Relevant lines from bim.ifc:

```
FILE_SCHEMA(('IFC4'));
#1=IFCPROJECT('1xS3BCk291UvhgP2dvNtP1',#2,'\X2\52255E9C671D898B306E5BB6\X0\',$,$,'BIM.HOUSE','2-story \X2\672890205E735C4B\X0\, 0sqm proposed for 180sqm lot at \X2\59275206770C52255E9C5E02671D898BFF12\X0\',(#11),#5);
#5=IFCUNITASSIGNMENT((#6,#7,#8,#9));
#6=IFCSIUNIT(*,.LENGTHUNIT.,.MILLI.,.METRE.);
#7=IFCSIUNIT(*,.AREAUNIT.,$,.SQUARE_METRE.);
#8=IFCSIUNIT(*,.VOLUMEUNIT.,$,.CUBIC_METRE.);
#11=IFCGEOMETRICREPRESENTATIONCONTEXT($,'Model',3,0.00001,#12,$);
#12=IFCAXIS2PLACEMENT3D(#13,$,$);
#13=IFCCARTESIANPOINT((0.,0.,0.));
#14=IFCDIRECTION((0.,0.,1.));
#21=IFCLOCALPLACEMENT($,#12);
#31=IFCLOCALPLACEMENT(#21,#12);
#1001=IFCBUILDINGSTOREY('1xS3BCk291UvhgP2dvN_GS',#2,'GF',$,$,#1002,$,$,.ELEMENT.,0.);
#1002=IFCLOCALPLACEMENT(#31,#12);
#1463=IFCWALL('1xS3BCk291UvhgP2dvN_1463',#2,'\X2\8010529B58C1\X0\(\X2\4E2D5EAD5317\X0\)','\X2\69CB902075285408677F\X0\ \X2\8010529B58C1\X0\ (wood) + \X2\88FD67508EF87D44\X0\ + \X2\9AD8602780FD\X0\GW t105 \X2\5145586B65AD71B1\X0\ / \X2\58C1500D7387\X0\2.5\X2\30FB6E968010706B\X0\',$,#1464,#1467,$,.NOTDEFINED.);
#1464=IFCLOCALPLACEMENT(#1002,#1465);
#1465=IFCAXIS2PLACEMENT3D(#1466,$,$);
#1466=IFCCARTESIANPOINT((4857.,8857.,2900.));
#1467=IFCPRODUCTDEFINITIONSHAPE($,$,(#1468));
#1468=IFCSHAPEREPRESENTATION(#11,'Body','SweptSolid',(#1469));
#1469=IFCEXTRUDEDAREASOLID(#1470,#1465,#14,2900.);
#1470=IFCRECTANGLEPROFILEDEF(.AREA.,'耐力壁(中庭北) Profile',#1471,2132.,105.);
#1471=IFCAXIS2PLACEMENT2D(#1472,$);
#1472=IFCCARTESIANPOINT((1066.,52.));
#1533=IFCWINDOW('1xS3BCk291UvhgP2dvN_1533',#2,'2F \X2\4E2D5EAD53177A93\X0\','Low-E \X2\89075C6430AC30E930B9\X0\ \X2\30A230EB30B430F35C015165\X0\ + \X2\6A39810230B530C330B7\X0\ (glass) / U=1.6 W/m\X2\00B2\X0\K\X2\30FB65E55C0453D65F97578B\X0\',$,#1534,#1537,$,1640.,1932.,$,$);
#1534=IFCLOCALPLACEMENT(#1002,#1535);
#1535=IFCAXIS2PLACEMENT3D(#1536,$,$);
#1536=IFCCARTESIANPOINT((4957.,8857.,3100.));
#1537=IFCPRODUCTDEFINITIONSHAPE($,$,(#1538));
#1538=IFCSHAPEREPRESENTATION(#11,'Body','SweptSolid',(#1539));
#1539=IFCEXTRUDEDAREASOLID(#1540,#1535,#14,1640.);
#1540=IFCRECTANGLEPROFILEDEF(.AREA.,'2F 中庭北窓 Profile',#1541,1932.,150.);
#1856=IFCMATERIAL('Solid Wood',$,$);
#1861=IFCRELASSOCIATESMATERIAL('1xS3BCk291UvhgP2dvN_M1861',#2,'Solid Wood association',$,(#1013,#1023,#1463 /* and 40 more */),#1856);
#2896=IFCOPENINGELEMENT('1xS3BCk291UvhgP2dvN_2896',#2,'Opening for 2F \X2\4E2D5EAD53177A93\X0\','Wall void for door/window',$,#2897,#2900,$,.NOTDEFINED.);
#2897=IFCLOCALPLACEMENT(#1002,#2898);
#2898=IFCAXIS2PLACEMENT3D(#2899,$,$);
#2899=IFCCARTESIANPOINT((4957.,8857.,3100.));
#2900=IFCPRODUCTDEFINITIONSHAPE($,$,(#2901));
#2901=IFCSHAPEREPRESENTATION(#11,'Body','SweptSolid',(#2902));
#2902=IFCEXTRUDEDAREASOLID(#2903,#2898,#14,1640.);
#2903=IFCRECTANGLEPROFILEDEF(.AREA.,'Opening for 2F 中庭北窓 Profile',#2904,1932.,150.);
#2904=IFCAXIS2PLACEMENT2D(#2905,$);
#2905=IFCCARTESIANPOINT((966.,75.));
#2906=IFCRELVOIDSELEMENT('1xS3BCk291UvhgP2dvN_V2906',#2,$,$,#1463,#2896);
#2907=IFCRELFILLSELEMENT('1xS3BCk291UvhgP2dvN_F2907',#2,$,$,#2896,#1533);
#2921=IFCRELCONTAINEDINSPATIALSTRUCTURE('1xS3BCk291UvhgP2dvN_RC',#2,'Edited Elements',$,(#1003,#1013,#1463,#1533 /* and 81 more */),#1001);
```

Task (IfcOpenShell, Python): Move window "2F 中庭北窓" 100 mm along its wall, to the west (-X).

```python
import ifcopenshell
import ifcopenshell.api.geometry
import ifcopenshell.util.placement
import ifcopenshell.util.unit

model = ifcopenshell.open("bim.ifc")
unit_scale = ifcopenshell.util.unit.calculate_unit_scale(model)

window = model.by_guid("1xS3BCk291UvhgP2dvN_1533")
opening = window.FillsVoids[0].RelatingOpeningElement
wall = opening.VoidsElements[0].RelatingBuildingElement

wall_matrix = ifcopenshell.util.placement.get_local_placement(wall.ObjectPlacement)
shift = wall_matrix[:3, 0] * -0.1 / unit_scale
before = ifcopenshell.util.placement.get_local_placement(window.ObjectPlacement)[:3, 3].copy()

# The window is not placed relative to its opening, so move both.
for product in (opening, window):
    matrix = ifcopenshell.util.placement.get_local_placement(product.ObjectPlacement)
    matrix[:3, 3] += shift
    ifcopenshell.api.geometry.edit_object_placement(model, product=product, matrix=matrix, is_si=False)

after = ifcopenshell.util.placement.get_local_placement(window.ObjectPlacement)[:3, 3]
print("window moved by", (after - before).round(3) + 0.0)

model.write("bim_edited.ifc")
```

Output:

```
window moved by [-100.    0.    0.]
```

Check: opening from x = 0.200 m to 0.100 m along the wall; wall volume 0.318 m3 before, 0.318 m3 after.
